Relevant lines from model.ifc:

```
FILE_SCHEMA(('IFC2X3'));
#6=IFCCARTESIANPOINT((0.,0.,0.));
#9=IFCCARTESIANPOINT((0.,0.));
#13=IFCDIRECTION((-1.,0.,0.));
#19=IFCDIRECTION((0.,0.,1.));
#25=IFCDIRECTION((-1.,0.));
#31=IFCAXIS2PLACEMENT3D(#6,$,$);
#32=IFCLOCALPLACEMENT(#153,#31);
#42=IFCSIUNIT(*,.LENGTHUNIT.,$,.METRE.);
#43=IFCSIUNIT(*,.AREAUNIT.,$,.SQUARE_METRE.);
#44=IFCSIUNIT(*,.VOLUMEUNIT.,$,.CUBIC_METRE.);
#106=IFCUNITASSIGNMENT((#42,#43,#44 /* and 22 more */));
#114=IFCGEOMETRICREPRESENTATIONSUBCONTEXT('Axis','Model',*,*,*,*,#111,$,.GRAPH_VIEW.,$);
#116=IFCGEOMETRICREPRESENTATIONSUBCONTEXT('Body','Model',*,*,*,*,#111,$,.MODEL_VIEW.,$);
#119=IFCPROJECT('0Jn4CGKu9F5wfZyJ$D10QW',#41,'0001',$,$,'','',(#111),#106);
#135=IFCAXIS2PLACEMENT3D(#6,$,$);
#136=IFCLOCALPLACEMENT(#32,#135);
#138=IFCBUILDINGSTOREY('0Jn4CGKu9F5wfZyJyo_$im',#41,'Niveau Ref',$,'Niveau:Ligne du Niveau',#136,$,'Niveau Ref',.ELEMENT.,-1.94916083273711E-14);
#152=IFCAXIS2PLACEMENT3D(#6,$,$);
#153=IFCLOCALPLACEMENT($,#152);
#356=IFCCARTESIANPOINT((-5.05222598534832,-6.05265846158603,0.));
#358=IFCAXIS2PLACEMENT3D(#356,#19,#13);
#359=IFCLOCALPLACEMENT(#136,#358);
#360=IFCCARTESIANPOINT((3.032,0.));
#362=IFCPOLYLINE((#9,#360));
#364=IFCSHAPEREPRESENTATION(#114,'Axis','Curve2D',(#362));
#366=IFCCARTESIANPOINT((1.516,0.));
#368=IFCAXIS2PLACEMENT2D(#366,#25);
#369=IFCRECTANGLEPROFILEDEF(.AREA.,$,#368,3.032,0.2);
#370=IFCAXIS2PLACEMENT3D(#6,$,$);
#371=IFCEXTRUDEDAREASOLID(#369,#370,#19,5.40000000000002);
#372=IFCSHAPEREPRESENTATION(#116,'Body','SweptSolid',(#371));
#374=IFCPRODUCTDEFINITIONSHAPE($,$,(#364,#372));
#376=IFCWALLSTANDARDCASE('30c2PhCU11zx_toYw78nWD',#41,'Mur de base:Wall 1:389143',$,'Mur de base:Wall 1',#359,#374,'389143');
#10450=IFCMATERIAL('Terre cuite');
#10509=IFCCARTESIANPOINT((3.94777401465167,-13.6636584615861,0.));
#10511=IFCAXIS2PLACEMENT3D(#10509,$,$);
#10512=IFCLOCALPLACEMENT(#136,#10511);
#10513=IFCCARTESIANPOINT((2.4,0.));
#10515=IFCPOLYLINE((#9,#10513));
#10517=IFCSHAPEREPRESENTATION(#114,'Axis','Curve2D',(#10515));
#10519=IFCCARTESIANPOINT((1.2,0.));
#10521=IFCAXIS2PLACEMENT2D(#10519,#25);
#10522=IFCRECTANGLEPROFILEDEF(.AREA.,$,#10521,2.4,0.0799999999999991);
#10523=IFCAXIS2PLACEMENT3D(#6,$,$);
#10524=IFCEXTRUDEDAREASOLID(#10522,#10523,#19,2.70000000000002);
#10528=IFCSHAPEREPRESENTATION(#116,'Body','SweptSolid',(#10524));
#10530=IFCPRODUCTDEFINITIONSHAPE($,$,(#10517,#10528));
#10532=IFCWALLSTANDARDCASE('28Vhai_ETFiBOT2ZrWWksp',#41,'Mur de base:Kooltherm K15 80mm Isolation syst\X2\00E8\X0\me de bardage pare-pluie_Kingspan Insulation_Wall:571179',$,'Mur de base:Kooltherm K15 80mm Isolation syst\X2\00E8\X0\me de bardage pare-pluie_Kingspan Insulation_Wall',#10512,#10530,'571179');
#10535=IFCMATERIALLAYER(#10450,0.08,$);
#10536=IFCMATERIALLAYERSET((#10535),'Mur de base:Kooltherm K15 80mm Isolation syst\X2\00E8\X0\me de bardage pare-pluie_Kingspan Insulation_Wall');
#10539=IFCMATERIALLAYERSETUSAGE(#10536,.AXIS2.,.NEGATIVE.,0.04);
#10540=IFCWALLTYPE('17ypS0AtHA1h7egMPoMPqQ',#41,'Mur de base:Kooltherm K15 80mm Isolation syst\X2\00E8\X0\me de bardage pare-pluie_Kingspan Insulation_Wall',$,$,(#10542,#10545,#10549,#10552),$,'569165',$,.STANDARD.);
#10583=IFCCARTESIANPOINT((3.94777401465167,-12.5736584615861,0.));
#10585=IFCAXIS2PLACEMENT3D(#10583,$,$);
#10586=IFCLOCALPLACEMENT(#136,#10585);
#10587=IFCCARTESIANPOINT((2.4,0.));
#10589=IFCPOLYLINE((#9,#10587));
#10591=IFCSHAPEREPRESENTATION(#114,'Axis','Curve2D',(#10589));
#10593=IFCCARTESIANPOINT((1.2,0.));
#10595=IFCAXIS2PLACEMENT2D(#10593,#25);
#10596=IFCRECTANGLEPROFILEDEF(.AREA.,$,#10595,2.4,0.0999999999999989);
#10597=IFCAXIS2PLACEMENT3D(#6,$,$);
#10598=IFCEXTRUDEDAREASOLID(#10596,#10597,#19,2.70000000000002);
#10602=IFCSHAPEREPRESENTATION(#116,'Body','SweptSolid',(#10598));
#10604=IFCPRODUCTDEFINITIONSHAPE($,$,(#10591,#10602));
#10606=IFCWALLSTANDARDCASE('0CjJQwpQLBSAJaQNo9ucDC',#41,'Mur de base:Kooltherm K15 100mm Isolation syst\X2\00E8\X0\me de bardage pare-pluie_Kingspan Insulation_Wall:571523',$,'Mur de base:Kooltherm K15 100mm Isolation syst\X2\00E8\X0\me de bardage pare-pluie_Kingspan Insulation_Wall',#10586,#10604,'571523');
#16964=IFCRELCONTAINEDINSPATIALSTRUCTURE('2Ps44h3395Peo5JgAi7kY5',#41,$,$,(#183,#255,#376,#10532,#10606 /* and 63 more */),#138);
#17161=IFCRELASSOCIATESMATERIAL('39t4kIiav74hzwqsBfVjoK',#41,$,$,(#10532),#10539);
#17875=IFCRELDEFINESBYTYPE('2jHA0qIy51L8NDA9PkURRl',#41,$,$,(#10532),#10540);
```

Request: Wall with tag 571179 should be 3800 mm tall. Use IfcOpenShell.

```python
import ifcopenshell
import ifcopenshell.geom
import ifcopenshell.util.representation
import ifcopenshell.util.shape

model = ifcopenshell.open("model.ifc")
settings = ifcopenshell.geom.settings()


def volume(element):
    """Net volume in cubic metres, openings subtracted."""
    shape = ifcopenshell.geom.create_shape(settings, element)
    return ifcopenshell.util.shape.get_volume(shape.geometry)


wall = model.by_guid("28Vhai_ETFiBOT2ZrWWksp")
before = volume(wall)

body = ifcopenshell.util.representation.get_representation(wall, "Model", "Body")
solid = body.Items[0]
old_height = solid.Depth
solid.Depth = 3.8
after = volume(wall)

print(f"height {old_height:g} -> {solid.Depth:g}, volume {before:.3f} -> {after:.3f} m3")

model.write("model_v2.ifc")
```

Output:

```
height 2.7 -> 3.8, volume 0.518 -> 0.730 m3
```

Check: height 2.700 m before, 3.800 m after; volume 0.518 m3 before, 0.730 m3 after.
